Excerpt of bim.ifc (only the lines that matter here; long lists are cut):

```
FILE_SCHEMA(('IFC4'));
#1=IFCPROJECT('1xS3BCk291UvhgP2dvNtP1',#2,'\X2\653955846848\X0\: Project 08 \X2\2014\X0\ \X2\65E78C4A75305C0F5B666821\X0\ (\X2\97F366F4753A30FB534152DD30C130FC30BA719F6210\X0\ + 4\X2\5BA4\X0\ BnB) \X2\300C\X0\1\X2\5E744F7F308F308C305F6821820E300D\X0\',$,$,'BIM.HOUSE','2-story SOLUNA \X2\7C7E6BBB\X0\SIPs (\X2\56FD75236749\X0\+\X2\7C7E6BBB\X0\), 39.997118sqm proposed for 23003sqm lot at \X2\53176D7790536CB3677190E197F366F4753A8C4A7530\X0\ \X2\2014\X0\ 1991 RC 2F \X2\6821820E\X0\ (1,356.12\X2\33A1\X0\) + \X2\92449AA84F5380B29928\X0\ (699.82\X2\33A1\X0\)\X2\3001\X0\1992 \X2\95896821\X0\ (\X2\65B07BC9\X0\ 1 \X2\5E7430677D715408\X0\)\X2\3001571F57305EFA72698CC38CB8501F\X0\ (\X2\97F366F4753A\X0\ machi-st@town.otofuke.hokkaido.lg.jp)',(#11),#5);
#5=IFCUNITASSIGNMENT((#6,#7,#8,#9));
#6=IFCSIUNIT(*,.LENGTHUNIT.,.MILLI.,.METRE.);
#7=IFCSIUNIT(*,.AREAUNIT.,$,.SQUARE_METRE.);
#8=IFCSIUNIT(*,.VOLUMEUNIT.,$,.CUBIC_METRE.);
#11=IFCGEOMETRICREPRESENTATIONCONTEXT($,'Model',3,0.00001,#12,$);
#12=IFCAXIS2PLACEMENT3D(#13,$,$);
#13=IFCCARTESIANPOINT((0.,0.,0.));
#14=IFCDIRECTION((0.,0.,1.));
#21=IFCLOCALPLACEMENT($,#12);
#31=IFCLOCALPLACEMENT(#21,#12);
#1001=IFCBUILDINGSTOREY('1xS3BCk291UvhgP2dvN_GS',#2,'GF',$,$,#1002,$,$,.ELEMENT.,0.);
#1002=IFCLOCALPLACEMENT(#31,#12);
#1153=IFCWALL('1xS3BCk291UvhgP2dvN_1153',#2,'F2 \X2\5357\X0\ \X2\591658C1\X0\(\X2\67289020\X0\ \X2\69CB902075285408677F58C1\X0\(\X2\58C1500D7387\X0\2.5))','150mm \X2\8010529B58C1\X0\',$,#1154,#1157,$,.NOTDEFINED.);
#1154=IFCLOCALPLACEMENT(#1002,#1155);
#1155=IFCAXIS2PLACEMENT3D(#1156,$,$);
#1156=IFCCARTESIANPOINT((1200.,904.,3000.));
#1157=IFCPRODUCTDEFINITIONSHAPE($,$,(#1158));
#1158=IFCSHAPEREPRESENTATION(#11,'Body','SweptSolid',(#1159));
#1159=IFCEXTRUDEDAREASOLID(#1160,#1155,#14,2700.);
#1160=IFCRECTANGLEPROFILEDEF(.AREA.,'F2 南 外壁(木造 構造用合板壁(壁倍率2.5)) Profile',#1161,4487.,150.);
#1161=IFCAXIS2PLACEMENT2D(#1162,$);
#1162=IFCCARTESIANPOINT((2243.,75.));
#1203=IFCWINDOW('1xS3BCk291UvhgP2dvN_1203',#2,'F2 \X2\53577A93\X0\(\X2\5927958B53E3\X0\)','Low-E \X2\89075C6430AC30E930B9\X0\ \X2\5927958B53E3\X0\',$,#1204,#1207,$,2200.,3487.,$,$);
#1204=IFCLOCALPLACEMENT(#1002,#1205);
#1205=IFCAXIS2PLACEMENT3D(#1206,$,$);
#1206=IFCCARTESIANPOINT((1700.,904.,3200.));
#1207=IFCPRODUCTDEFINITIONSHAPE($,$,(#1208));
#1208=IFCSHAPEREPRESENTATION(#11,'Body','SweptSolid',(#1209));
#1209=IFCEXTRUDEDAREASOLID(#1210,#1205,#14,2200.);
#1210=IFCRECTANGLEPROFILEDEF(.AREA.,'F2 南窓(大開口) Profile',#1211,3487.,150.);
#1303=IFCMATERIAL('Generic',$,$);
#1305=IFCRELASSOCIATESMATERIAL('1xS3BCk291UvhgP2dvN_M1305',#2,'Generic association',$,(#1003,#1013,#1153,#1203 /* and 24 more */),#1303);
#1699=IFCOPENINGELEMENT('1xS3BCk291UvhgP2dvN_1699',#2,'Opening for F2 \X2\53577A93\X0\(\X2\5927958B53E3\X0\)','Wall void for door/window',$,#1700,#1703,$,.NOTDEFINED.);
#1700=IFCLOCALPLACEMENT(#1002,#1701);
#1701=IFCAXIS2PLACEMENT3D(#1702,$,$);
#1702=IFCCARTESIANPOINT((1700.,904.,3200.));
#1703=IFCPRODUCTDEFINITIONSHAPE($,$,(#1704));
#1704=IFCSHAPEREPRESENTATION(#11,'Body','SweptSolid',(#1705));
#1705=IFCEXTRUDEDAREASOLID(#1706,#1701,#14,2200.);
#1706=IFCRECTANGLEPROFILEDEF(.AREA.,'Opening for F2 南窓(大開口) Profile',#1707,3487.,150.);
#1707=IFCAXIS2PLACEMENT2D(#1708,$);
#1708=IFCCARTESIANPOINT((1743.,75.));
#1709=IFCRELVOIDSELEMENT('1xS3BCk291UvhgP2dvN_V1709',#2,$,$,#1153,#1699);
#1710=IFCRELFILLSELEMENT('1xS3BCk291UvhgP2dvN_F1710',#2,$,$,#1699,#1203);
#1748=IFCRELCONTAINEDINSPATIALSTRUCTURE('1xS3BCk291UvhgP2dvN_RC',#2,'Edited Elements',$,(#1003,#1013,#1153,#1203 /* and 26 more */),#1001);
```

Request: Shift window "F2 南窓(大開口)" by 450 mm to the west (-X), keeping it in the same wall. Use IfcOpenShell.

```python
import ifcopenshell
import ifcopenshell.api.geometry
import ifcopenshell.util.placement
import ifcopenshell.util.unit

model = ifcopenshell.open("bim.ifc")
unit_scale = ifcopenshell.util.unit.calculate_unit_scale(model)

window = model.by_guid("1xS3BCk291UvhgP2dvN_1203")
opening = window.FillsVoids[0].RelatingOpeningElement
wall = opening.VoidsElements[0].RelatingBuildingElement

wall_matrix = ifcopenshell.util.placement.get_local_placement(wall.ObjectPlacement)
shift = wall_matrix[:3, 0] * -0.45 / unit_scale
before = ifcopenshell.util.placement.get_local_placement(window.ObjectPlacement)[:3, 3].copy()

# The window is not placed relative to its opening, so move both.
for product in (opening, window):
    matrix = ifcopenshell.util.placement.get_local_placement(product.ObjectPlacement)
    matrix[:3, 3] += shift
    ifcopenshell.api.geometry.edit_object_placement(model, product=product, matrix=matrix, is_si=False)

after = ifcopenshell.util.placement.get_local_placement(window.ObjectPlacement)[:3, 3]
print("window moved by", (after - before).round(3) + 0.0)

model.write("bim-out.ifc")
```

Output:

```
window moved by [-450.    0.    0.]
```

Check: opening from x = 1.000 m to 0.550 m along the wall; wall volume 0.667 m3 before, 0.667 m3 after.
